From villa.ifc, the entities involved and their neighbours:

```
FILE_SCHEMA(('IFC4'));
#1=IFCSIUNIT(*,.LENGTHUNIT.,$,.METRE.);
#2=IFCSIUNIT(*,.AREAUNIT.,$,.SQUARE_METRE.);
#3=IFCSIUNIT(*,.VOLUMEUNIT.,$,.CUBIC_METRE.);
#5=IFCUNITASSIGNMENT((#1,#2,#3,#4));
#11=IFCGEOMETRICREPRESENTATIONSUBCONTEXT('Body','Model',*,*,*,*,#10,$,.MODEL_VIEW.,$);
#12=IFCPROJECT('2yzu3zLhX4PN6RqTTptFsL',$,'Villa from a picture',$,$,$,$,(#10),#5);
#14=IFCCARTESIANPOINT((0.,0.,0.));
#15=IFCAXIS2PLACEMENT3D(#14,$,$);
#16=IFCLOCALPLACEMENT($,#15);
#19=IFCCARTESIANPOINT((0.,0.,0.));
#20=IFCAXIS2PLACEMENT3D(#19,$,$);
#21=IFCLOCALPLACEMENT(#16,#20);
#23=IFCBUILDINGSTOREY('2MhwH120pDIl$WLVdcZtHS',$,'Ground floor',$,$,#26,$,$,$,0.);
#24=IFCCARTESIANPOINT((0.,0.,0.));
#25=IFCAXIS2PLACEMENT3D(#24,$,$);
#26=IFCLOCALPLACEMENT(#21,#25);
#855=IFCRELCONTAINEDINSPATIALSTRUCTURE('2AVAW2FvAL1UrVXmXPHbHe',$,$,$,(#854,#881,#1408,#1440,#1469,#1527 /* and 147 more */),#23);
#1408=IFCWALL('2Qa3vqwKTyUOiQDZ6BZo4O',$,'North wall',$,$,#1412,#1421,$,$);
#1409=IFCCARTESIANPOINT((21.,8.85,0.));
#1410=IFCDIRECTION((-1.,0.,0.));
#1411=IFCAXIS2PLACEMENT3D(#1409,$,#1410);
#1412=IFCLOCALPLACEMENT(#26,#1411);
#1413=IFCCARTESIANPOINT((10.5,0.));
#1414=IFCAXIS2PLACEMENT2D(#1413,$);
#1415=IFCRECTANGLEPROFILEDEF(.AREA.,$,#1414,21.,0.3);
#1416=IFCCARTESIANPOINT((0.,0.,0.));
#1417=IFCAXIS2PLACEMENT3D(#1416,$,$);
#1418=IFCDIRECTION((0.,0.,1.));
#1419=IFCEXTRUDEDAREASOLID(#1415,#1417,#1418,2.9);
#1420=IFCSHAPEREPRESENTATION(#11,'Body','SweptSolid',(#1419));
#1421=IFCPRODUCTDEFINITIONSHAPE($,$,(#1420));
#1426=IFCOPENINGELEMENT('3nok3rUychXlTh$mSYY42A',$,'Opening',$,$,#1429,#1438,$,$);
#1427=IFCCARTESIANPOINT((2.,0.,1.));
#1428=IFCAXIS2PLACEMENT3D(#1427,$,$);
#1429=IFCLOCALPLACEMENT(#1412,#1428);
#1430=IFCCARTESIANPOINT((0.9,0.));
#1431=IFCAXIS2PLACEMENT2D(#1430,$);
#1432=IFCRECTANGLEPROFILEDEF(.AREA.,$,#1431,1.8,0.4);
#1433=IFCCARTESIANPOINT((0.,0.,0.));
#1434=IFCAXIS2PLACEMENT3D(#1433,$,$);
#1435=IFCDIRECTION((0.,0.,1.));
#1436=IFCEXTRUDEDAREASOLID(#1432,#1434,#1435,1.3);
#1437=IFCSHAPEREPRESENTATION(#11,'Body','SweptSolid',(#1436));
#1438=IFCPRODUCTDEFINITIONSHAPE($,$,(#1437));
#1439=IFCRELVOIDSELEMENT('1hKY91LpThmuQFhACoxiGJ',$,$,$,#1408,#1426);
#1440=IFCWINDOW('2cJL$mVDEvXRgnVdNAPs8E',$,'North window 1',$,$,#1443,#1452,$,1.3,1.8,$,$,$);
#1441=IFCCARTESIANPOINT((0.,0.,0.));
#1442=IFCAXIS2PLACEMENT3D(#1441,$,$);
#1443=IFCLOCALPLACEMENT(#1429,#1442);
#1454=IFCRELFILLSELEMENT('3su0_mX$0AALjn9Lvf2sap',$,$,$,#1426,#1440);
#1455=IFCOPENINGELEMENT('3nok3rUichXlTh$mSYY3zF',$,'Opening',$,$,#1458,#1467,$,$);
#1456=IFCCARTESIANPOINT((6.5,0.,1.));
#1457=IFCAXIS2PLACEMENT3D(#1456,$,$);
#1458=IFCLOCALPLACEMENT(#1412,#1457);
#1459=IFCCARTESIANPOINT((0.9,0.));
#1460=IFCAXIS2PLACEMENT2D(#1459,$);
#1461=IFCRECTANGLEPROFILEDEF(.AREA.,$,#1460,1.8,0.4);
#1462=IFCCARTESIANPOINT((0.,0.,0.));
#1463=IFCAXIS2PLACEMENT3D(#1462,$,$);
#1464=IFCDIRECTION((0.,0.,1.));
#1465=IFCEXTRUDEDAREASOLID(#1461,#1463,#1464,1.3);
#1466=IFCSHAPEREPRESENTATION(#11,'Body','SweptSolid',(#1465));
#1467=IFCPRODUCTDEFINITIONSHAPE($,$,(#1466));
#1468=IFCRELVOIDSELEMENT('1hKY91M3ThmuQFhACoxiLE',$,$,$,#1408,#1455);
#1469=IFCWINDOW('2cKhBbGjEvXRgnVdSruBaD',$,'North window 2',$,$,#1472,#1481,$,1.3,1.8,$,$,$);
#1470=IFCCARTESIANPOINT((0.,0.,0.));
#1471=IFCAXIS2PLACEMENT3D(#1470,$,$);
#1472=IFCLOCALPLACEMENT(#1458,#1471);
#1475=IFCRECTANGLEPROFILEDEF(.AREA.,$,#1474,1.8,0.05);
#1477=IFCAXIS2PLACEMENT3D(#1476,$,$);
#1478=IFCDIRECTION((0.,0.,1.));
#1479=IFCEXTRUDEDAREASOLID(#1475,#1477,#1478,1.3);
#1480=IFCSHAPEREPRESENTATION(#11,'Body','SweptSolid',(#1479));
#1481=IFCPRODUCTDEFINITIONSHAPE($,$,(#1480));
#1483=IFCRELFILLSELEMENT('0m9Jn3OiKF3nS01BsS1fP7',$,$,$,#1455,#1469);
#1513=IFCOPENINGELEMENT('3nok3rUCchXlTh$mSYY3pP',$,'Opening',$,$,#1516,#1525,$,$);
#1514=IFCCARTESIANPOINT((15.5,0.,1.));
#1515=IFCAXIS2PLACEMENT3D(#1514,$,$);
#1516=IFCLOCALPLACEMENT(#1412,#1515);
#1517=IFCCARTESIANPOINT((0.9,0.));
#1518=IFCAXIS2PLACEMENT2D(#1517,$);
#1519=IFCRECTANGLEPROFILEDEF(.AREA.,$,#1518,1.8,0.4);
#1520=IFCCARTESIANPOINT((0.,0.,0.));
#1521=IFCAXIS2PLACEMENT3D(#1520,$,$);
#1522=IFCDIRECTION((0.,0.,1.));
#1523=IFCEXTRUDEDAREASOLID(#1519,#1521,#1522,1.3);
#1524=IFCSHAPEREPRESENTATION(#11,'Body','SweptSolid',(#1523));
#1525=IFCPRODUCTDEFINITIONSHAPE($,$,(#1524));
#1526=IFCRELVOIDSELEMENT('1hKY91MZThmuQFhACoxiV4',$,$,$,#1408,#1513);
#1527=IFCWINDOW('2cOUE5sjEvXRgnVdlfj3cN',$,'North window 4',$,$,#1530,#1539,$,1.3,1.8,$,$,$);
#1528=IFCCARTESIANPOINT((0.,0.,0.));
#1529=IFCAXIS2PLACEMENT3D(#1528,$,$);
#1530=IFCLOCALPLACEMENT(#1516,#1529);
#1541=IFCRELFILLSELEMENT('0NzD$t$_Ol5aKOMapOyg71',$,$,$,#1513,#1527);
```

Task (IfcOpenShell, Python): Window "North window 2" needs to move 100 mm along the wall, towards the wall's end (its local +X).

```python
import ifcopenshell
import ifcopenshell.api.geometry
import ifcopenshell.util.placement
import ifcopenshell.util.unit

model = ifcopenshell.open("villa.ifc")
unit_scale = ifcopenshell.util.unit.calculate_unit_scale(model)

window = model.by_id(1469)
opening = window.FillsVoids[0].RelatingOpeningElement
wall = opening.VoidsElements[0].RelatingBuildingElement

wall_matrix = ifcopenshell.util.placement.get_local_placement(wall.ObjectPlacement)
shift = wall_matrix[:3, 0] * 0.1 / unit_scale
before = ifcopenshell.util.placement.get_local_placement(window.ObjectPlacement)[:3, 3].copy()

# The window is placed relative to its opening, so it follows when the opening moves.
matrix = ifcopenshell.util.placement.get_local_placement(opening.ObjectPlacement)
matrix[:3, 3] += shift
ifcopenshell.api.geometry.edit_object_placement(
    model, product=opening, matrix=matrix, is_si=False, should_transform_children=True
)

after = ifcopenshell.util.placement.get_local_placement(window.ObjectPlacement)[:3, 3]
print("window moved by", (after - before).round(3) + 0.0)

model.write("villa_v2.ifc")
```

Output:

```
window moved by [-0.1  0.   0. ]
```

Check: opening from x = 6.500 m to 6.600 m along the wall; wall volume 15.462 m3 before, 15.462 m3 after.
